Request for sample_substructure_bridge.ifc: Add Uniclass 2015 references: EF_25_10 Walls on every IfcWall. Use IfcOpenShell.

First a look at what the model holds.

```python
import ifcopenshell

model = ifcopenshell.open("sample_substructure_bridge.ifc")
print(model.schema)
print("classifications:", [c.Name for c in model.by_type("IfcClassification")])
for ifc_class in ("IfcDoor", "IfcRoof", "IfcStair", "IfcWall", "IfcWindow"):
    print(ifc_class, len(model.by_type(ifc_class)))
```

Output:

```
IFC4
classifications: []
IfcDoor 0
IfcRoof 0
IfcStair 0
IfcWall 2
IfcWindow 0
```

```python
import ifcopenshell
import ifcopenshell.api.classification

model = ifcopenshell.open("sample_substructure_bridge.ifc")

system = ifcopenshell.api.classification.add_classification(model, classification="Uniclass 2015")

codes = {
    "IfcWall": ("EF_25_10", "Walls"),
}
for ifc_class, (code, name) in codes.items():
    products = model.by_type(ifc_class)
    ifcopenshell.api.classification.add_reference(
        model, products=products, classification=system, identification=code, name=name
    )
    print(code, len(products))

model.write("sample_substructure_bridge_updated.ifc")
```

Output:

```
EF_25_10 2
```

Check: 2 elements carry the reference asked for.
